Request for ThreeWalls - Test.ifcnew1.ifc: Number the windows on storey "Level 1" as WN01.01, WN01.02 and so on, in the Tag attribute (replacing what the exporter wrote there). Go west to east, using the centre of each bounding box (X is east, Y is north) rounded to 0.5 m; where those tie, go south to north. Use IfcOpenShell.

First a look at what the model holds.

```python
import ifcopenshell
import ifcopenshell.util.element
import ifcopenshell.util.placement

model = ifcopenshell.open("ThreeWalls - Test.ifcnew1.ifc")
print(model.schema)
storey = next(s for s in model.by_type("IfcBuildingStorey") if s.Name == "Level 1")
windows = [e for e in ifcopenshell.util.element.get_decomposition(storey) if e.is_a("IfcWindow")]
for e in sorted(windows, key=lambda e: e.id()):
    origin = ifcopenshell.util.placement.get_local_placement(e.ObjectPlacement)[:3, 3]
    print(e.id(), e.Tag, e.Name, origin.round(2) + 0.0, sep=" | ")
```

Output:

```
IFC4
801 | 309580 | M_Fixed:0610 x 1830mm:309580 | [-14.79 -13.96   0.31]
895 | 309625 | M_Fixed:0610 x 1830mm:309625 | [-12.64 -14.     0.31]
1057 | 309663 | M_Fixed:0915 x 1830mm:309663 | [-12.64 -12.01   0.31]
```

```python
import ifcopenshell
import ifcopenshell.geom
import ifcopenshell.util.element
import ifcopenshell.util.shape

model = ifcopenshell.open("ThreeWalls - Test.ifcnew1.ifc")
settings = ifcopenshell.geom.settings()
settings.set("use-world-coords", True)


def centre(element):
    shape = ifcopenshell.geom.create_shape(settings, element)
    return ifcopenshell.util.shape.get_bbox_centroid(shape.geometry)


storey = next(s for s in model.by_type("IfcBuildingStorey") if s.Name == "Level 1")
windows = [e for e in ifcopenshell.util.element.get_decomposition(storey) if e.is_a("IfcWindow")]

# Insertion points can sit at a corner or the storey origin, so sort by the geometry (in metres).
centres = {e: centre(e) for e in windows}
windows.sort(key=lambda e: (round(centres[e][0] / 0.5), centres[e][1]))

for i, e in enumerate(windows, start=1):
    number = f"WN01.{i:02d}"
    e.Tag = number
    print(e.id(), number)

model.write("ThreeWalls - Test.ifcnew1_v2.ifc")
```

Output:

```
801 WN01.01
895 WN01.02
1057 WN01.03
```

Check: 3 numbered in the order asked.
